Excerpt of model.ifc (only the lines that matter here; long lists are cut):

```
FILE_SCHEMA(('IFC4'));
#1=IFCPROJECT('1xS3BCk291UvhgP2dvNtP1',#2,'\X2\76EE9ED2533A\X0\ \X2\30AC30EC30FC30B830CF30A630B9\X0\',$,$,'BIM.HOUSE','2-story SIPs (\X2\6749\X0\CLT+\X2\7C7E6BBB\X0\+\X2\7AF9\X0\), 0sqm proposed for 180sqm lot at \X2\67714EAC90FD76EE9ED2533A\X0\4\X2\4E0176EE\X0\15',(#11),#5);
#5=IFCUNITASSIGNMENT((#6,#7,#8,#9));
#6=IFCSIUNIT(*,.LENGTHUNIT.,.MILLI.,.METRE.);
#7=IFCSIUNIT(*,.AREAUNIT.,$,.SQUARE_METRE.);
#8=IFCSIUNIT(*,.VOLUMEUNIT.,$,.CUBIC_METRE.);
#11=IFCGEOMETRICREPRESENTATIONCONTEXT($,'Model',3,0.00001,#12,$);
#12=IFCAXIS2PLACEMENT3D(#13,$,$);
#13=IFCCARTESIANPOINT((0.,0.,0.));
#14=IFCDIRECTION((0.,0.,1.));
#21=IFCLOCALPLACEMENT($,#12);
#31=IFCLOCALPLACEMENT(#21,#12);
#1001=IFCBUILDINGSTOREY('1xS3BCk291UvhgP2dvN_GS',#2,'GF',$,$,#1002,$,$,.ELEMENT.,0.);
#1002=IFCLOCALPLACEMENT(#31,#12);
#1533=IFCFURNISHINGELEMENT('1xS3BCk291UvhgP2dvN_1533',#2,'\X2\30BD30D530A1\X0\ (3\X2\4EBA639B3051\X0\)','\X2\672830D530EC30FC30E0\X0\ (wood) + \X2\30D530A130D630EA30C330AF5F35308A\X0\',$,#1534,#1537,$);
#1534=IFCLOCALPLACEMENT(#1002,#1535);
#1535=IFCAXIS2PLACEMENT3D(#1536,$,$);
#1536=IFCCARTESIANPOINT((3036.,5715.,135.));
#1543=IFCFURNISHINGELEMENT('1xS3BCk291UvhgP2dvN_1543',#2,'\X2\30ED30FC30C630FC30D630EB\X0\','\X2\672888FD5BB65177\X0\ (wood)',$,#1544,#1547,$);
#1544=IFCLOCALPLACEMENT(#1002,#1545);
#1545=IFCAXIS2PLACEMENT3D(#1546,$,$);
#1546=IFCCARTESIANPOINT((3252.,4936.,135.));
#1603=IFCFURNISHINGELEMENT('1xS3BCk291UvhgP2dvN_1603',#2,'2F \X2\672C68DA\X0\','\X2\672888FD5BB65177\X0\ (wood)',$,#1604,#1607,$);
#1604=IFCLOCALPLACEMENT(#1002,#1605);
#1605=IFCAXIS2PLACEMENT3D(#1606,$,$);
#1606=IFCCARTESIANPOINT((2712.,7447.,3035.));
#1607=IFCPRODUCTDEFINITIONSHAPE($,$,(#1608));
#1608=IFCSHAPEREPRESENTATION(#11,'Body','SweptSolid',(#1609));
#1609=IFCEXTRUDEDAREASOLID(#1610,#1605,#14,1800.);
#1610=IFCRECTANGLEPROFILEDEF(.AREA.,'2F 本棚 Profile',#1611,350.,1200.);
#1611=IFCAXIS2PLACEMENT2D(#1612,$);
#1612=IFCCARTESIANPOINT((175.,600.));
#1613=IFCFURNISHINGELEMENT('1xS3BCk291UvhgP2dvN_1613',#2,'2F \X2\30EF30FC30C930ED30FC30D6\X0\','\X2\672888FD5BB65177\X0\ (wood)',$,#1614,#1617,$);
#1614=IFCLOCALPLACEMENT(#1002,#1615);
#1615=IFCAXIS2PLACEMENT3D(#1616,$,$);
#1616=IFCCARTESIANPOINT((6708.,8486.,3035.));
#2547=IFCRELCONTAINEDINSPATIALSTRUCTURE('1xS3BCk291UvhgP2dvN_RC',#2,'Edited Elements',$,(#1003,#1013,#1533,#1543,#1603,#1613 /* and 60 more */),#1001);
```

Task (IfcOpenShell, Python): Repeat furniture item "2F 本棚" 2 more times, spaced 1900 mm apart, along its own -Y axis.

```python
import ifcopenshell
import ifcopenshell.api.geometry
import ifcopenshell.api.root
import ifcopenshell.util.element
import ifcopenshell.util.placement

model = ifcopenshell.open("model.ifc")


def reuse_history(source, copy):
    """copy_class also copies each property set's owner history, people and application; keep the originals."""
    for rel in copy.IsDefinedBy:
        if rel.is_a("IfcRelDefinesByProperties") and (history := rel.RelatingPropertyDefinition.OwnerHistory):
            rel.RelatingPropertyDefinition.OwnerHistory = source.OwnerHistory
            ifcopenshell.util.element.remove_deep2(model, history)


source = model.by_guid("1xS3BCk291UvhgP2dvN_1603")
base = ifcopenshell.util.placement.get_local_placement(source.ObjectPlacement)
step = -base[:3, 1] * 1900.0

for i in range(1, 3):
    copy = ifcopenshell.api.root.copy_class(model, product=source)
    copy.Representation = ifcopenshell.util.element.copy_deep(
        model, source.Representation, exclude=["IfcGeometricRepresentationContext", "IfcRepresentationMap"]
    )
    reuse_history(source, copy)
    matrix = base.copy()
    matrix[:3, 3] += i * step
    print("added at", matrix[:3, 3].round(3) + 0.0)
    ifcopenshell.api.geometry.edit_object_placement(model, product=copy, matrix=matrix, is_si=False)

model.write("model_rev.ifc")
```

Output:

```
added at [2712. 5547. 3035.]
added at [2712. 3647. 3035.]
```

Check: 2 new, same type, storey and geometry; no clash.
